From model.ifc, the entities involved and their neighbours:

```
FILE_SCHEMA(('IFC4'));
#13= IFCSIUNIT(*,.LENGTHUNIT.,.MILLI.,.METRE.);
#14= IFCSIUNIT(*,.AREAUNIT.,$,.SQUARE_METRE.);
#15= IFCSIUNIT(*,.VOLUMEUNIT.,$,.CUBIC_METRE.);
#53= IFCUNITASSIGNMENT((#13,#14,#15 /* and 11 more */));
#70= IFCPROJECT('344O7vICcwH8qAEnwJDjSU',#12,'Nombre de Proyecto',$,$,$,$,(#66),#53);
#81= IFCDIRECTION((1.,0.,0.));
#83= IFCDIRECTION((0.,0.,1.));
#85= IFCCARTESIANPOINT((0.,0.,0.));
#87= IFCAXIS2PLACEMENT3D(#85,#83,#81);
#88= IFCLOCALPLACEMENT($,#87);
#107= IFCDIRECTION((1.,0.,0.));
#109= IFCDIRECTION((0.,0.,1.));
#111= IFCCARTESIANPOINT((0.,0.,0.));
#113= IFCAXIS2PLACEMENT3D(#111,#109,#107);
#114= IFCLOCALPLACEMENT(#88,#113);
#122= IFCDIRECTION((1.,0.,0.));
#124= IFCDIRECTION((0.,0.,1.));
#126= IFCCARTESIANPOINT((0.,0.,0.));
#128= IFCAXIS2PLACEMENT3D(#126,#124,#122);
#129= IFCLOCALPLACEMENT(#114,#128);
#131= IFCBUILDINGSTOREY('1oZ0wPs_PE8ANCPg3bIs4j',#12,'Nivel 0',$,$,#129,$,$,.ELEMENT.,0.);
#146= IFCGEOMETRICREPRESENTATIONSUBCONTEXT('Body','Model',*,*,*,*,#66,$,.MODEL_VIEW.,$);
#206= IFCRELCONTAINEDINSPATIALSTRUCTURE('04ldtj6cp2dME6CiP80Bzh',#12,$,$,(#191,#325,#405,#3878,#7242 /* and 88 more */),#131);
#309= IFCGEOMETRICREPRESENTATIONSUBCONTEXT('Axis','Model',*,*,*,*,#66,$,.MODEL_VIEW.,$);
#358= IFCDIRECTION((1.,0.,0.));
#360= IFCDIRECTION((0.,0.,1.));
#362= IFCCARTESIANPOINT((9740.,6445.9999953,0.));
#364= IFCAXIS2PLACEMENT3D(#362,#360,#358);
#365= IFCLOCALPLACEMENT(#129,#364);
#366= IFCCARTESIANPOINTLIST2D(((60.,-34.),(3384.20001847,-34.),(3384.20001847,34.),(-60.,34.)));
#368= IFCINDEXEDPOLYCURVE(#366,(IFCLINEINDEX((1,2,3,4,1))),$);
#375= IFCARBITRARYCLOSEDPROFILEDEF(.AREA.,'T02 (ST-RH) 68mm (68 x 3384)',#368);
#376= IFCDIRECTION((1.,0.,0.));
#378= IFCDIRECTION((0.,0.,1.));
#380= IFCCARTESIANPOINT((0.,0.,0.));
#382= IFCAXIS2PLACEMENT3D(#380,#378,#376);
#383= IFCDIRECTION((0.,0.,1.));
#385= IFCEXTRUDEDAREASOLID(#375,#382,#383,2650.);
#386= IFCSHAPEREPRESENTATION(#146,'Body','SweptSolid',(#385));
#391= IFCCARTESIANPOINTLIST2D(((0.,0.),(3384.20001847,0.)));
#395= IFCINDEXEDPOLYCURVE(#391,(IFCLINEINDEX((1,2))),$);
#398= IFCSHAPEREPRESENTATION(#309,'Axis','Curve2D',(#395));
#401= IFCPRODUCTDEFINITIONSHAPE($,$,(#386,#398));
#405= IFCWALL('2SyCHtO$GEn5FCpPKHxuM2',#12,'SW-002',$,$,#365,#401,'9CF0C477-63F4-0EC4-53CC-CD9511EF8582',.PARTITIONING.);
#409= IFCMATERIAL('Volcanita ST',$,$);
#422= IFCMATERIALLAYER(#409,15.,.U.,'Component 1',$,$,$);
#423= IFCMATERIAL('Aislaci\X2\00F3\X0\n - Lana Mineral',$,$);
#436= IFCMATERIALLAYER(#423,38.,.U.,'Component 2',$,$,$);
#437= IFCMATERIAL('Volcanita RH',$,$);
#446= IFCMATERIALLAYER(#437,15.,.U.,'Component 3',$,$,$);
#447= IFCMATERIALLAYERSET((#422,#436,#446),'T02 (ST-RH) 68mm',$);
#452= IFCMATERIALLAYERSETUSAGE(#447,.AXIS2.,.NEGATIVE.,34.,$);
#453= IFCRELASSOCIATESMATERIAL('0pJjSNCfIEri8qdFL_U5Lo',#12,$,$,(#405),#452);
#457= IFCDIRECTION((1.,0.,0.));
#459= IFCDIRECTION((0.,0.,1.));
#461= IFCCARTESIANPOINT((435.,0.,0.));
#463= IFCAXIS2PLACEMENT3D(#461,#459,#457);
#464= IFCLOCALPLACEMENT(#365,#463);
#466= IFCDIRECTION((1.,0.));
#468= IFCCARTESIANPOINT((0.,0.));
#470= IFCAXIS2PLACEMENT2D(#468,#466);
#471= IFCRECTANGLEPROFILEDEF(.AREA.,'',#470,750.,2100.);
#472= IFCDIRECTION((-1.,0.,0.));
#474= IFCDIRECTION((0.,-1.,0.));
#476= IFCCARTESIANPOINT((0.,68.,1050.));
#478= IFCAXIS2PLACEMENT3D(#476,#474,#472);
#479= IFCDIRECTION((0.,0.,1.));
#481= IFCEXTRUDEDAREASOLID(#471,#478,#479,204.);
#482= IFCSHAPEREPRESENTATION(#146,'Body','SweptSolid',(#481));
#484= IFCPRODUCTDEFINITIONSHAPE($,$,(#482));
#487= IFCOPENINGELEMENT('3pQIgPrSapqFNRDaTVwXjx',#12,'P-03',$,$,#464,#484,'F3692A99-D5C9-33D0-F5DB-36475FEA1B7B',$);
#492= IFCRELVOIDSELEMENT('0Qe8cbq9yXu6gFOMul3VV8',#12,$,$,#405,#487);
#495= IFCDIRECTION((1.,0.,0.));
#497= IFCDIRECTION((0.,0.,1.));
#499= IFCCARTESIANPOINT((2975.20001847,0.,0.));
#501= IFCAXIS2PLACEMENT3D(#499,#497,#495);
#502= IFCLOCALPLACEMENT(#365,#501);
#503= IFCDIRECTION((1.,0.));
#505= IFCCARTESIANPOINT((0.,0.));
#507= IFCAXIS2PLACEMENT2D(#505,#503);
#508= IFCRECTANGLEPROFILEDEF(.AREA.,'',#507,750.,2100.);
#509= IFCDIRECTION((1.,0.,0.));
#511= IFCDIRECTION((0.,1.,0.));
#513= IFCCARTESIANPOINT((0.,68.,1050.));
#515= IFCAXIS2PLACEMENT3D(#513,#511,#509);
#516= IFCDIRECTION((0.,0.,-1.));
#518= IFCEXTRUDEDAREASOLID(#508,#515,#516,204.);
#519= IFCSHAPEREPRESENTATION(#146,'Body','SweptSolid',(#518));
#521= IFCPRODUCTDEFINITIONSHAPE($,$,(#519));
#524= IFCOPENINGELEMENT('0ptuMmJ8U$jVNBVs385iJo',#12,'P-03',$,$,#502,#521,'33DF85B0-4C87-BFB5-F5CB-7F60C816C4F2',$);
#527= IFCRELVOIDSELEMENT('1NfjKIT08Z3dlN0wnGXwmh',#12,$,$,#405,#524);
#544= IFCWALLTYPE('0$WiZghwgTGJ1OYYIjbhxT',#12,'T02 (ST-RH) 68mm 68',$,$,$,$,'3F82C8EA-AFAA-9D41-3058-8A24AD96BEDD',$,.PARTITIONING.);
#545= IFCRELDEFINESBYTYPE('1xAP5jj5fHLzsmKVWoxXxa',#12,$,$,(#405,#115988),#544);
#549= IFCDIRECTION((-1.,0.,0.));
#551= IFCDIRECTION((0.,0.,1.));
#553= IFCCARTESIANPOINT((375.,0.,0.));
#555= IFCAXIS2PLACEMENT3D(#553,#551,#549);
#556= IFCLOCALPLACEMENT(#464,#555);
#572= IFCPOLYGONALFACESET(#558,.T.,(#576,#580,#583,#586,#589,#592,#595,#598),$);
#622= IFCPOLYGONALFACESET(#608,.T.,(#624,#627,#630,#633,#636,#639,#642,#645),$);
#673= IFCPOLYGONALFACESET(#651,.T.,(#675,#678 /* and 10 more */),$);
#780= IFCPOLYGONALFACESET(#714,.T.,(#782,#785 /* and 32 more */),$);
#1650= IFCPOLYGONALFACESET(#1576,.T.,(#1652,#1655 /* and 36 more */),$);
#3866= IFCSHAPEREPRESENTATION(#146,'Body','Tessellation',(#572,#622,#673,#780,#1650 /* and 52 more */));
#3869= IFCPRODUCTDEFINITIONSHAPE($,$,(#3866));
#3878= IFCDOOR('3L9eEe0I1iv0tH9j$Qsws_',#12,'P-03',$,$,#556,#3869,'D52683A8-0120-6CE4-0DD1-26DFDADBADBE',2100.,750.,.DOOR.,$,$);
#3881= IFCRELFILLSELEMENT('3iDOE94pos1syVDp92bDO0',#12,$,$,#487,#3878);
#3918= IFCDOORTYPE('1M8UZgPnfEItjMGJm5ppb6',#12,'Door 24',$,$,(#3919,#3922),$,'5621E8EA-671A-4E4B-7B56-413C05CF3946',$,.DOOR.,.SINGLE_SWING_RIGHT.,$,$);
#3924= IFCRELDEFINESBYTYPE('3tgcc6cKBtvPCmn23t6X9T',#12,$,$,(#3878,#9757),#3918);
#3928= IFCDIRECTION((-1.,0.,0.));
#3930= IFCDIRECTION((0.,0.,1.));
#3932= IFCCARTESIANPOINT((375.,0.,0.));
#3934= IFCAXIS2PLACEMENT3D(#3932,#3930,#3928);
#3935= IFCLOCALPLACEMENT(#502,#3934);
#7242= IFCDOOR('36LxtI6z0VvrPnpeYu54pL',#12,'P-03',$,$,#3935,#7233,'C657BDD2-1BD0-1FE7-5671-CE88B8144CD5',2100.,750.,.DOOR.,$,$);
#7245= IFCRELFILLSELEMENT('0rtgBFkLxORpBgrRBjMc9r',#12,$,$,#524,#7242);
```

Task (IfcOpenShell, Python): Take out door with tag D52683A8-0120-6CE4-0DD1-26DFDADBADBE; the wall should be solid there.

```python
import ifcopenshell
import ifcopenshell.api.feature
import ifcopenshell.api.root
import ifcopenshell.geom
import ifcopenshell.util.shape

model = ifcopenshell.open("model.ifc")
settings = ifcopenshell.geom.settings()


def volume(element):
    """Net volume in cubic metres, openings subtracted."""
    shape = ifcopenshell.geom.create_shape(settings, element)
    return ifcopenshell.util.shape.get_volume(shape.geometry)


door = model.by_id(3878)
opening = door.FillsVoids[0].RelatingOpeningElement
wall = opening.VoidsElements[0].RelatingBuildingElement
before = volume(wall)

ifcopenshell.api.root.remove_product(model, product=door)
ifcopenshell.api.feature.remove_feature(model, feature=opening)

after = volume(wall)

print(f"wall volume {before:.3f} -> {after:.3f} m3")

model.write("model_edited.ifc")
```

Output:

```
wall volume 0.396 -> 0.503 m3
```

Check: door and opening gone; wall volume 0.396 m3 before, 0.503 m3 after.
